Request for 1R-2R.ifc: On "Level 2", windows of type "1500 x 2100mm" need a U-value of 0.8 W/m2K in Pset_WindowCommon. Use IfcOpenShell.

First a look at what the model holds.

```python
import ifcopenshell
import ifcopenshell.util.element

model = ifcopenshell.open("1R-2R.ifc")
print(model.schema)
storey = next(s for s in model.by_type("IfcBuildingStorey") if s.Name == "Level 2")
windows = [e for e in ifcopenshell.util.element.get_decomposition(storey) if e.is_a("IfcWindow")]
seen = {}
for e in windows:
    element_type = ifcopenshell.util.element.get_type(e)
    key = (element_type.Name if element_type != e and element_type else None, ifcopenshell.util.element.get_pset(e, "Pset_WindowCommon", "ThermalTransmittance"))
    seen[key] = seen.get(key, 0) + 1
for (name, value), count in sorted(seen.items(), key=str):
    print(count, "x", name, "|", value)
```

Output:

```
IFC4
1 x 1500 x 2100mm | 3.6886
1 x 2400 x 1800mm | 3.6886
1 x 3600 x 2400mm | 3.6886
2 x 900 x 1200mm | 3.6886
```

```python
import ifcopenshell
import ifcopenshell.api.pset
import ifcopenshell.util.element

model = ifcopenshell.open("1R-2R.ifc")

storey = next(s for s in model.by_type("IfcBuildingStorey") if s.Name == "Level 2")
windows = [e for e in ifcopenshell.util.element.get_decomposition(storey) if e.is_a("IfcWindow")]

count = 0
for e in windows:
    element_type = ifcopenshell.util.element.get_type(e)
    if element_type in (None, e) or element_type.Name != "1500 x 2100mm":
        continue
    # add_pset returns the element's existing set when there is one.
    pset = ifcopenshell.api.pset.add_pset(model, product=e, name="Pset_WindowCommon")
    ifcopenshell.api.pset.edit_pset(model, pset=pset, properties={"ThermalTransmittance": 0.8})
    count += 1

print(count, "windows updated")

model.write("1R-2R-out.ifc")
```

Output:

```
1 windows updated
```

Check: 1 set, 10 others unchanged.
